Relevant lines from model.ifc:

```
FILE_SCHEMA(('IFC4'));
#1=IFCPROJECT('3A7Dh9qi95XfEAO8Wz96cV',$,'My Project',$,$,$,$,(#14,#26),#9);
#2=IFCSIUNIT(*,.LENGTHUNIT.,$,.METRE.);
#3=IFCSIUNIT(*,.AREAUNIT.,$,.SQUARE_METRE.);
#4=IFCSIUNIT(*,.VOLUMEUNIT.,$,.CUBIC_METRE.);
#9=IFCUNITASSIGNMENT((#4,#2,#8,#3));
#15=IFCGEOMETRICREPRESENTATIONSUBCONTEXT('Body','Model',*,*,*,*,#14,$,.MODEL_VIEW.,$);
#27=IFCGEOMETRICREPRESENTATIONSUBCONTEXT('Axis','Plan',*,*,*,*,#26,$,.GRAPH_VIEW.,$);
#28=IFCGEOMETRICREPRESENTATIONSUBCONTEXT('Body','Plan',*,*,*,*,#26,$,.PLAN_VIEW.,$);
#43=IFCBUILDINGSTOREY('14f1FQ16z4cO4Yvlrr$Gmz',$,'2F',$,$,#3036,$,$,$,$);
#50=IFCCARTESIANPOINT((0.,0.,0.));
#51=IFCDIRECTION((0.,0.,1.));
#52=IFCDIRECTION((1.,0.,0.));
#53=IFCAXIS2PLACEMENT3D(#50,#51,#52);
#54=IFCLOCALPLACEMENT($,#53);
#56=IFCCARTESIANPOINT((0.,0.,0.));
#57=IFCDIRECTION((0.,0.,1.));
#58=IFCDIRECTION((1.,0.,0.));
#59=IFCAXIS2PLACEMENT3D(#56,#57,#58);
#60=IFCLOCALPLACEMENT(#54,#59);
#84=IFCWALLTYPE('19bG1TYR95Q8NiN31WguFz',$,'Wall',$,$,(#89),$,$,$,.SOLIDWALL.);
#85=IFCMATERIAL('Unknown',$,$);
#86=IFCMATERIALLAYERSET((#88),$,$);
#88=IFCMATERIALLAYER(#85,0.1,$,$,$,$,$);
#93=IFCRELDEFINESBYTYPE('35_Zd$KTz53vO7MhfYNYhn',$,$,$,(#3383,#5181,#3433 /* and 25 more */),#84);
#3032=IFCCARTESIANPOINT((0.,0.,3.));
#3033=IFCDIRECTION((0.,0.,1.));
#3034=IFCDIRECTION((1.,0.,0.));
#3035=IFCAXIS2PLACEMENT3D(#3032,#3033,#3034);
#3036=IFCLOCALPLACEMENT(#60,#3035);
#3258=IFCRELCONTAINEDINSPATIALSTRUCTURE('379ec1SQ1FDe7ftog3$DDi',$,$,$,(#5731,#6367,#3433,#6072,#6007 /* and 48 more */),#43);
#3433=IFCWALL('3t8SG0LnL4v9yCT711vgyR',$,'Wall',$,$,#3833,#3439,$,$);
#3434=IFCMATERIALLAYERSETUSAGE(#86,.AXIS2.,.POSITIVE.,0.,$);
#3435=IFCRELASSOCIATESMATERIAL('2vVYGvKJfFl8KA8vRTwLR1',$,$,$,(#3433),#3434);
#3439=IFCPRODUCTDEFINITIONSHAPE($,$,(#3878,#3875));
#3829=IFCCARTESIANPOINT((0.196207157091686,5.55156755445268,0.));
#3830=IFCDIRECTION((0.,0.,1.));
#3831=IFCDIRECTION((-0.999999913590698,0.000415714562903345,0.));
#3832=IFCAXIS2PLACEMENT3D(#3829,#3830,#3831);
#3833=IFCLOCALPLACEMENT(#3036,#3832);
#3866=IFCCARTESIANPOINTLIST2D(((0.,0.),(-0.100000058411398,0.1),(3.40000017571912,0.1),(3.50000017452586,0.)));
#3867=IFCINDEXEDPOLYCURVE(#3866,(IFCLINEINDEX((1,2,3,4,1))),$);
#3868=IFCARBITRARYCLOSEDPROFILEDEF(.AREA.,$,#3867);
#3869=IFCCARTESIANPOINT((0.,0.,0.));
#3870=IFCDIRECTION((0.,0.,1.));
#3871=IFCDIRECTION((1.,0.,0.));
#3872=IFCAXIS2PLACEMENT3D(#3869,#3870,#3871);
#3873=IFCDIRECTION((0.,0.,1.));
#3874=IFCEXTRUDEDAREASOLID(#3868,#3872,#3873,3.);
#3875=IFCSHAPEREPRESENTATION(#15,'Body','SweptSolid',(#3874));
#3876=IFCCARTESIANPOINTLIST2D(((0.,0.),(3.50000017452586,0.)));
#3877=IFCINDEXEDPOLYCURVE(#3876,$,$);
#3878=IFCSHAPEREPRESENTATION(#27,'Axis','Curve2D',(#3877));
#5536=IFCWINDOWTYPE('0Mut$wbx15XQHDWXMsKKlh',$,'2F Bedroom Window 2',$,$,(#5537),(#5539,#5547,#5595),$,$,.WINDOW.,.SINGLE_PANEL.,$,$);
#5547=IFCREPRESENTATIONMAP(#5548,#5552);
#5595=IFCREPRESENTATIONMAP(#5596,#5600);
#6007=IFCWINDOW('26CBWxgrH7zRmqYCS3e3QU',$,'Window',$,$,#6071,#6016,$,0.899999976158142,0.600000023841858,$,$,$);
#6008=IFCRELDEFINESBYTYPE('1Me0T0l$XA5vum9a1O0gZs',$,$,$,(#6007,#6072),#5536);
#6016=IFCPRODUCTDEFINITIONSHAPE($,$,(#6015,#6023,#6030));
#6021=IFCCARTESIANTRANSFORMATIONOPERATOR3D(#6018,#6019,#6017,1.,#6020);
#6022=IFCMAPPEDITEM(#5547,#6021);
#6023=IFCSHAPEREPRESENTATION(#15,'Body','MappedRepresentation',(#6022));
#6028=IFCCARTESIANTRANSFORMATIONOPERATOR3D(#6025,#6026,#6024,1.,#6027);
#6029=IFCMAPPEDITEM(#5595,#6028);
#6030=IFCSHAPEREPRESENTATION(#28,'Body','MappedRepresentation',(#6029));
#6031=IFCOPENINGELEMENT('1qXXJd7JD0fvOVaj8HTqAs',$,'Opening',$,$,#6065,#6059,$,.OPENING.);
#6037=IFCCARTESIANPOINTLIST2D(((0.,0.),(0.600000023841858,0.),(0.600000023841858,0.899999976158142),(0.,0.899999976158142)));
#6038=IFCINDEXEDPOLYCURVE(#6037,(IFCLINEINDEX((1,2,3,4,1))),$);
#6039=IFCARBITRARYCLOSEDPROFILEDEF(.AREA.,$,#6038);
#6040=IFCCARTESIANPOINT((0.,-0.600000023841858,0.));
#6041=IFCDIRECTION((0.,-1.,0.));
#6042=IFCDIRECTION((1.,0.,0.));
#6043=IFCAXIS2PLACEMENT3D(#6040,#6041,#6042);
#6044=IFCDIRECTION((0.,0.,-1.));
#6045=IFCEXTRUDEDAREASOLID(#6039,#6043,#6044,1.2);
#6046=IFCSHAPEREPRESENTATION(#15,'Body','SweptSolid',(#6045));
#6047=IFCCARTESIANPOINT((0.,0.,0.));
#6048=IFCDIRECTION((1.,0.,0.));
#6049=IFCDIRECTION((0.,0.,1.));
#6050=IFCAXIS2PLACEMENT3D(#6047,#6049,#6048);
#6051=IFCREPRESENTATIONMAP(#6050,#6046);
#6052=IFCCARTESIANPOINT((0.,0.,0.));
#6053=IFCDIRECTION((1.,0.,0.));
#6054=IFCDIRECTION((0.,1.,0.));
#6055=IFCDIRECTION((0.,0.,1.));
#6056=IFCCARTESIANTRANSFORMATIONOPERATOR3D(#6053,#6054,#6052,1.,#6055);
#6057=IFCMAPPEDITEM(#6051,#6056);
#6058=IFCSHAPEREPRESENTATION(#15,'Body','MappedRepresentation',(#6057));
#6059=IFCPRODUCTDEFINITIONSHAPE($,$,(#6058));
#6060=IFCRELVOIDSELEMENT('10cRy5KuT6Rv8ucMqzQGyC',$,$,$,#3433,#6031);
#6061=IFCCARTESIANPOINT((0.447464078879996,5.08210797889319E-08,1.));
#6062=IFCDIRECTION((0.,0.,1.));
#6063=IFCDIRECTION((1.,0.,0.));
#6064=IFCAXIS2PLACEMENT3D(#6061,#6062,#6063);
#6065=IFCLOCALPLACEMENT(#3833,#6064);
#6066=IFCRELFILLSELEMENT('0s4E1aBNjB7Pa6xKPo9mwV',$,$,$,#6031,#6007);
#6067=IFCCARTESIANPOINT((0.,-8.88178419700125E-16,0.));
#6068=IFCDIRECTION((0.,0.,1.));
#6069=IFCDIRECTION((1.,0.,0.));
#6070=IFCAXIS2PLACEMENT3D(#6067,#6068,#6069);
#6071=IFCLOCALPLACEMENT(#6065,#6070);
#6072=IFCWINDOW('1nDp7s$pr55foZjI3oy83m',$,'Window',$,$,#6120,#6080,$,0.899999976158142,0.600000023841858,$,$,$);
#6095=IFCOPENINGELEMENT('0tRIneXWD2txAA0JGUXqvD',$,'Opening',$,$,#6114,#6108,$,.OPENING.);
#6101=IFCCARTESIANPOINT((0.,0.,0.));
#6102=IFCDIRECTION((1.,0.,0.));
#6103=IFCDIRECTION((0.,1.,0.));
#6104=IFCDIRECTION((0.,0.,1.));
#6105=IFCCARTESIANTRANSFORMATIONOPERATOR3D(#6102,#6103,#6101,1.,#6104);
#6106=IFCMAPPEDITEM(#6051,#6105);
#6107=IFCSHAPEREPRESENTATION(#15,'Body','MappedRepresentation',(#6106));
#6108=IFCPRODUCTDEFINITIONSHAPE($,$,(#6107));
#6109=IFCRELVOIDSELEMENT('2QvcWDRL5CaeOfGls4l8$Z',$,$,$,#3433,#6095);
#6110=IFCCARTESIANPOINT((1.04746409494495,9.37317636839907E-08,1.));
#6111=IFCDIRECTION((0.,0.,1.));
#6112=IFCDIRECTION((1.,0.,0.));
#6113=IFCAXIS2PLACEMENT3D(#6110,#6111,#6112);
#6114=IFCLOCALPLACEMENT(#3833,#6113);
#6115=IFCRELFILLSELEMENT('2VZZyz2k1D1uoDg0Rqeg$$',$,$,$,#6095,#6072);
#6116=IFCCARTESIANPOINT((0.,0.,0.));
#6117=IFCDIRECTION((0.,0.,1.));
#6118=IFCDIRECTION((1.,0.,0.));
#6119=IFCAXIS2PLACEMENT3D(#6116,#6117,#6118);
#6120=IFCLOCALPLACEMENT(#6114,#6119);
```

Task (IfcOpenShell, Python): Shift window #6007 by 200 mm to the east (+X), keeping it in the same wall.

```python
import ifcopenshell
import ifcopenshell.api.geometry
import ifcopenshell.util.placement

model = ifcopenshell.open("model.ifc")

window = model.by_id(6007)
opening = window.FillsVoids[0].RelatingOpeningElement
wall = opening.VoidsElements[0].RelatingBuildingElement

wall_matrix = ifcopenshell.util.placement.get_local_placement(wall.ObjectPlacement)
shift = wall_matrix[:3, 0] * -0.2
before = ifcopenshell.util.placement.get_local_placement(window.ObjectPlacement)[:3, 3].copy()

# The window is placed relative to its opening, so it follows when the opening moves.
matrix = ifcopenshell.util.placement.get_local_placement(opening.ObjectPlacement)
matrix[:3, 3] += shift
ifcopenshell.api.geometry.edit_object_placement(
    model, product=opening, matrix=matrix, is_si=False, should_transform_children=True
)

after = ifcopenshell.util.placement.get_local_placement(window.ObjectPlacement)[:3, 3]
print("window moved by", (after - before).round(3) + 0.0)

model.write("model_v2.ifc")
```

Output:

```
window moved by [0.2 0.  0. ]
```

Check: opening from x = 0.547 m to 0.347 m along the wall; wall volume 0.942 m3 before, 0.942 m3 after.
